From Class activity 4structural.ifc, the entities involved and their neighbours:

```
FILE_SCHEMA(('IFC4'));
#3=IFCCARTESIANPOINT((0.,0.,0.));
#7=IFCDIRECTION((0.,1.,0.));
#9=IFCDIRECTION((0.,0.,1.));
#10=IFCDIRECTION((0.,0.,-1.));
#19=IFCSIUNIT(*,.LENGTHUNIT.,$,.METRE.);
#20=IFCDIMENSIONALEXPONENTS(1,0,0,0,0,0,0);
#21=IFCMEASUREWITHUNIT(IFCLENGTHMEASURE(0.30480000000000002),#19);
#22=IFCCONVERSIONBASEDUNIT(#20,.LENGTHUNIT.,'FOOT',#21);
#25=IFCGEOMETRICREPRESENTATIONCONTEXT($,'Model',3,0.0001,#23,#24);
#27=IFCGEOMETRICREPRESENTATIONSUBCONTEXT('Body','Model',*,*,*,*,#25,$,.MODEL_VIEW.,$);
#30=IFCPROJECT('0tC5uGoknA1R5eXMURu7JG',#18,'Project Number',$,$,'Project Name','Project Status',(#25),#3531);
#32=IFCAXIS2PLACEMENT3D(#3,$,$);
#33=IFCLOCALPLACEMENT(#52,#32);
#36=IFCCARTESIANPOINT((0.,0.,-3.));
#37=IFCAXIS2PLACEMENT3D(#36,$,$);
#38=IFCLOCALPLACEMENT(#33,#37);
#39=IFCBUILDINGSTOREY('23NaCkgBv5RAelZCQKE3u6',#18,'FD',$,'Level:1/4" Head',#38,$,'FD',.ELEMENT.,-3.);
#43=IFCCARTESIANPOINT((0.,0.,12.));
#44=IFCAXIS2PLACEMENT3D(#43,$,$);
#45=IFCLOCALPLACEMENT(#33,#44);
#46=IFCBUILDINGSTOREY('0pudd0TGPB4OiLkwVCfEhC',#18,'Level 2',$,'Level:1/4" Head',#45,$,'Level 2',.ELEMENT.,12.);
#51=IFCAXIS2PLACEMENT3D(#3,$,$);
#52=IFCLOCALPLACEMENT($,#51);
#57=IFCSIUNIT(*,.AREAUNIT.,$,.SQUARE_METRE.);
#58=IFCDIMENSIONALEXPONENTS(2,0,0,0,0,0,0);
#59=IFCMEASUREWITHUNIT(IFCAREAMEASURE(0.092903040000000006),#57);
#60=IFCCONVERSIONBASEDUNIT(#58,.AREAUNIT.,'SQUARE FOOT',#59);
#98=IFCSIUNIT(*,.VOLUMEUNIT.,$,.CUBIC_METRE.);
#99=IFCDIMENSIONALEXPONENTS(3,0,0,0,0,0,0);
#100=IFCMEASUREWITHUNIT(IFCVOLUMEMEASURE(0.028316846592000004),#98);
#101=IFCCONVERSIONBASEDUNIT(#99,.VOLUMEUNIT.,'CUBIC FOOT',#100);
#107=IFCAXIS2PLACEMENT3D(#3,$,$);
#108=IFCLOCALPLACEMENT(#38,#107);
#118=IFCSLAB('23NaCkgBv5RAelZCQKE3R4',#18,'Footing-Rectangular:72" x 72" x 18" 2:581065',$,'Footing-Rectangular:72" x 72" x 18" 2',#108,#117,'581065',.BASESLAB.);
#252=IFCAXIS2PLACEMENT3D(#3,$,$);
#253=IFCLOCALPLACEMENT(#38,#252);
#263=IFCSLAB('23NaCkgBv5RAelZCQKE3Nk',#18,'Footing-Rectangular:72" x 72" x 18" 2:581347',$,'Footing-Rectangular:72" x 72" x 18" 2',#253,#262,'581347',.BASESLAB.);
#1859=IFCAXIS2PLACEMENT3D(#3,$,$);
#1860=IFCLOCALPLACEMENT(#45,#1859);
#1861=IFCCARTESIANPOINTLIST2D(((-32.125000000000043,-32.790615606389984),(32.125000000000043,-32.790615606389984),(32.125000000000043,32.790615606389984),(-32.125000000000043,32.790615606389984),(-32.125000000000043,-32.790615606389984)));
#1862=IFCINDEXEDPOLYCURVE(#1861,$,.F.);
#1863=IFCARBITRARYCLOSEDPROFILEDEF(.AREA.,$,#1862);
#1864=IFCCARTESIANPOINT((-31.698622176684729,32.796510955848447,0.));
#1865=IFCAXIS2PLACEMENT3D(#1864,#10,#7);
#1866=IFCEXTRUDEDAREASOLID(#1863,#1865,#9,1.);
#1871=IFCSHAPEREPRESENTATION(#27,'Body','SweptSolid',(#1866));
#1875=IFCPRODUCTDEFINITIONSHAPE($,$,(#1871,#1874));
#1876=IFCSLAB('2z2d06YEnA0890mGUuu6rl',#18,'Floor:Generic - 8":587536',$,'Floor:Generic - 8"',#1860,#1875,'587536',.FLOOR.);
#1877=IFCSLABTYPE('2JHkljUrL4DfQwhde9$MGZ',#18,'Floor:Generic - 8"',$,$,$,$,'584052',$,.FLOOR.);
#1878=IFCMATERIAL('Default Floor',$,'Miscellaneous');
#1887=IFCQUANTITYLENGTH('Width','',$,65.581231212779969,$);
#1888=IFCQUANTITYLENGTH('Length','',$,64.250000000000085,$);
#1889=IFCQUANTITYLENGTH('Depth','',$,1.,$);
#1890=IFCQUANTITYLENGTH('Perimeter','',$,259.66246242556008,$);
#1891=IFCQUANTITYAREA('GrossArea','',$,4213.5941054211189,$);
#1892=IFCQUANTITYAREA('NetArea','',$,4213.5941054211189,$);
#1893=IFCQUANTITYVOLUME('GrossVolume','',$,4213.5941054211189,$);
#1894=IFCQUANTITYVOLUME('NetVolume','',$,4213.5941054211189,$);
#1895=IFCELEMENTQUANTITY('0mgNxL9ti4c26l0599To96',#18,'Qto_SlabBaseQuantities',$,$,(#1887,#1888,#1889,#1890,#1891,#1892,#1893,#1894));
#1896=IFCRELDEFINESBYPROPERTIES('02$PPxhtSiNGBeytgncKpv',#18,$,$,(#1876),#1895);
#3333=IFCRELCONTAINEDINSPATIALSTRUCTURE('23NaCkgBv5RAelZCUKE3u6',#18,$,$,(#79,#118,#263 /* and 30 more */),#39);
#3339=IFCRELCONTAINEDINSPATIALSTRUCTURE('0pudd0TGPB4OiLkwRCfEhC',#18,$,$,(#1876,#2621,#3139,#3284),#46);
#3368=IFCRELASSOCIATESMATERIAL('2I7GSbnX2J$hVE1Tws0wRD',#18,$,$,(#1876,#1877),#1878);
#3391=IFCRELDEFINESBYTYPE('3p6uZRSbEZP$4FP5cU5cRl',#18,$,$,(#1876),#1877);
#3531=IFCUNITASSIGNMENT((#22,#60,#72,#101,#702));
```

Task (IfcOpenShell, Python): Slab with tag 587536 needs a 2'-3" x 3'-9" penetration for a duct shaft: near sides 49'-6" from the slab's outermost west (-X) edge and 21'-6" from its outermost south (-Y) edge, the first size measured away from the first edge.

```python
import numpy as np
import ifcopenshell
import ifcopenshell.api.feature
import ifcopenshell.api.geometry
import ifcopenshell.api.pset
import ifcopenshell.api.root
import ifcopenshell.geom
import ifcopenshell.util.element
import ifcopenshell.util.placement
import ifcopenshell.util.representation
import ifcopenshell.util.shape
import ifcopenshell.util.unit

model = ifcopenshell.open("Class activity 4structural.ifc")
unit_scale = ifcopenshell.util.unit.calculate_unit_scale(model)
area_scale = ifcopenshell.util.unit.calculate_unit_scale(model, "AREAUNIT")
volume_scale = ifcopenshell.util.unit.calculate_unit_scale(model, "VOLUMEUNIT")
settings = ifcopenshell.geom.settings()


def volume(element):
    """Net volume in cubic metres, openings subtracted."""
    shape = ifcopenshell.geom.create_shape(settings, element)
    return ifcopenshell.util.shape.get_volume(shape.geometry)


slab = model.by_guid("2z2d06YEnA0890mGUuu6rl")
before = volume(slab)

# Extent in the slab's own axes, in metres. The edges named are its -X and -Y sides.
slab_shape = ifcopenshell.geom.create_shape(settings, slab)
vertices = ifcopenshell.util.shape.get_vertices(slab_shape.geometry)
x_min, y_min, bottom = vertices.min(axis=0)
top = vertices[:, 2].max()

opening = ifcopenshell.api.root.create_entity(model, ifc_class="IfcOpeningElement", name="Duct shaft opening", predefined_type="OPENING")
context = ifcopenshell.util.representation.get_context(model, "Model", "Body", "MODEL_VIEW")
width, depth = 0.6858, 1.143
outline = [(0.0, 0.0), (width, 0.0), (width, depth), (0.0, depth), (0.0, 0.0)]
# Overshoot both faces by 50 mm so the cut is clean.
shape = ifcopenshell.api.geometry.add_slab_representation(
    model, context=context, depth=top - bottom + 0.1, polyline=outline
)
ifcopenshell.api.geometry.assign_representation(model, product=opening, representation=shape)

matrix = ifcopenshell.util.placement.get_local_placement(slab.ObjectPlacement)
matrix[:, 3] = matrix @ np.append(np.array([x_min + 15.0876, y_min + 6.5532, bottom - 0.05]) / unit_scale, 1.0)
ifcopenshell.api.geometry.edit_object_placement(model, product=opening, matrix=matrix, is_si=False)
ifcopenshell.api.feature.add_feature(model, feature=opening, element=slab)

after = volume(slab)

# Update the slab's stored quantities.
qto = model.by_id(ifcopenshell.util.element.get_pset(slab, "Qto_SlabBaseQuantities", should_inherit=False)["id"])
ifcopenshell.api.pset.edit_qto(model, qto=qto, properties={
    "NetArea": after / (top - bottom) / area_scale,
    "NetVolume": after / volume_scale,
})

print(f"slab volume {before:.3f} -> {after:.3f} m3")

model.write("Class activity 4structural_rev.ifc")
```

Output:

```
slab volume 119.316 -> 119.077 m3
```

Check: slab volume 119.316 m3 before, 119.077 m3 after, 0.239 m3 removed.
